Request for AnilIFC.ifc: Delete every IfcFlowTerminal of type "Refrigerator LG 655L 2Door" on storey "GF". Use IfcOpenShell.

First a look at what the model holds.

```python
import ifcopenshell
import ifcopenshell.util.element

model = ifcopenshell.open("AnilIFC.ifc")
print(model.schema)
storey = next(s for s in model.by_type("IfcBuildingStorey") if s.Name == "GF")
terminals = [e for e in ifcopenshell.util.element.get_decomposition(storey) if e.is_a("IfcFlowTerminal")]
seen = {}
for e in terminals:
    element_type = ifcopenshell.util.element.get_type(e)
    name = element_type.Name if element_type not in (None, e) else None
    seen[name] = seen.get(name, 0) + 1
for name, count in sorted(seen.items(), key=str):
    print(count, "x", name)
```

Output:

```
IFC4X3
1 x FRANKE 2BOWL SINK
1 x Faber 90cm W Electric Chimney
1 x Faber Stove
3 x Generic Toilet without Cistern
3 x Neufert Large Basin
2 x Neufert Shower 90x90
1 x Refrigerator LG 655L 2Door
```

```python
import ifcopenshell
import ifcopenshell.api.root
import ifcopenshell.util.element

model = ifcopenshell.open("AnilIFC.ifc")

storey = next(s for s in model.by_type("IfcBuildingStorey") if s.Name == "GF")
terminals = [e for e in ifcopenshell.util.element.get_decomposition(storey) if e.is_a("IfcFlowTerminal")]
targets = [e for e in terminals if (t := ifcopenshell.util.element.get_type(e)) not in (None, e) and t.Name == "Refrigerator LG 655L 2Door"]

for e in targets:
    ifcopenshell.api.root.remove_product(model, product=e)
print(len(targets), "removed")

model.write("AnilIFC_updated.ifc")
```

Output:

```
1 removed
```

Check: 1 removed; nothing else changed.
